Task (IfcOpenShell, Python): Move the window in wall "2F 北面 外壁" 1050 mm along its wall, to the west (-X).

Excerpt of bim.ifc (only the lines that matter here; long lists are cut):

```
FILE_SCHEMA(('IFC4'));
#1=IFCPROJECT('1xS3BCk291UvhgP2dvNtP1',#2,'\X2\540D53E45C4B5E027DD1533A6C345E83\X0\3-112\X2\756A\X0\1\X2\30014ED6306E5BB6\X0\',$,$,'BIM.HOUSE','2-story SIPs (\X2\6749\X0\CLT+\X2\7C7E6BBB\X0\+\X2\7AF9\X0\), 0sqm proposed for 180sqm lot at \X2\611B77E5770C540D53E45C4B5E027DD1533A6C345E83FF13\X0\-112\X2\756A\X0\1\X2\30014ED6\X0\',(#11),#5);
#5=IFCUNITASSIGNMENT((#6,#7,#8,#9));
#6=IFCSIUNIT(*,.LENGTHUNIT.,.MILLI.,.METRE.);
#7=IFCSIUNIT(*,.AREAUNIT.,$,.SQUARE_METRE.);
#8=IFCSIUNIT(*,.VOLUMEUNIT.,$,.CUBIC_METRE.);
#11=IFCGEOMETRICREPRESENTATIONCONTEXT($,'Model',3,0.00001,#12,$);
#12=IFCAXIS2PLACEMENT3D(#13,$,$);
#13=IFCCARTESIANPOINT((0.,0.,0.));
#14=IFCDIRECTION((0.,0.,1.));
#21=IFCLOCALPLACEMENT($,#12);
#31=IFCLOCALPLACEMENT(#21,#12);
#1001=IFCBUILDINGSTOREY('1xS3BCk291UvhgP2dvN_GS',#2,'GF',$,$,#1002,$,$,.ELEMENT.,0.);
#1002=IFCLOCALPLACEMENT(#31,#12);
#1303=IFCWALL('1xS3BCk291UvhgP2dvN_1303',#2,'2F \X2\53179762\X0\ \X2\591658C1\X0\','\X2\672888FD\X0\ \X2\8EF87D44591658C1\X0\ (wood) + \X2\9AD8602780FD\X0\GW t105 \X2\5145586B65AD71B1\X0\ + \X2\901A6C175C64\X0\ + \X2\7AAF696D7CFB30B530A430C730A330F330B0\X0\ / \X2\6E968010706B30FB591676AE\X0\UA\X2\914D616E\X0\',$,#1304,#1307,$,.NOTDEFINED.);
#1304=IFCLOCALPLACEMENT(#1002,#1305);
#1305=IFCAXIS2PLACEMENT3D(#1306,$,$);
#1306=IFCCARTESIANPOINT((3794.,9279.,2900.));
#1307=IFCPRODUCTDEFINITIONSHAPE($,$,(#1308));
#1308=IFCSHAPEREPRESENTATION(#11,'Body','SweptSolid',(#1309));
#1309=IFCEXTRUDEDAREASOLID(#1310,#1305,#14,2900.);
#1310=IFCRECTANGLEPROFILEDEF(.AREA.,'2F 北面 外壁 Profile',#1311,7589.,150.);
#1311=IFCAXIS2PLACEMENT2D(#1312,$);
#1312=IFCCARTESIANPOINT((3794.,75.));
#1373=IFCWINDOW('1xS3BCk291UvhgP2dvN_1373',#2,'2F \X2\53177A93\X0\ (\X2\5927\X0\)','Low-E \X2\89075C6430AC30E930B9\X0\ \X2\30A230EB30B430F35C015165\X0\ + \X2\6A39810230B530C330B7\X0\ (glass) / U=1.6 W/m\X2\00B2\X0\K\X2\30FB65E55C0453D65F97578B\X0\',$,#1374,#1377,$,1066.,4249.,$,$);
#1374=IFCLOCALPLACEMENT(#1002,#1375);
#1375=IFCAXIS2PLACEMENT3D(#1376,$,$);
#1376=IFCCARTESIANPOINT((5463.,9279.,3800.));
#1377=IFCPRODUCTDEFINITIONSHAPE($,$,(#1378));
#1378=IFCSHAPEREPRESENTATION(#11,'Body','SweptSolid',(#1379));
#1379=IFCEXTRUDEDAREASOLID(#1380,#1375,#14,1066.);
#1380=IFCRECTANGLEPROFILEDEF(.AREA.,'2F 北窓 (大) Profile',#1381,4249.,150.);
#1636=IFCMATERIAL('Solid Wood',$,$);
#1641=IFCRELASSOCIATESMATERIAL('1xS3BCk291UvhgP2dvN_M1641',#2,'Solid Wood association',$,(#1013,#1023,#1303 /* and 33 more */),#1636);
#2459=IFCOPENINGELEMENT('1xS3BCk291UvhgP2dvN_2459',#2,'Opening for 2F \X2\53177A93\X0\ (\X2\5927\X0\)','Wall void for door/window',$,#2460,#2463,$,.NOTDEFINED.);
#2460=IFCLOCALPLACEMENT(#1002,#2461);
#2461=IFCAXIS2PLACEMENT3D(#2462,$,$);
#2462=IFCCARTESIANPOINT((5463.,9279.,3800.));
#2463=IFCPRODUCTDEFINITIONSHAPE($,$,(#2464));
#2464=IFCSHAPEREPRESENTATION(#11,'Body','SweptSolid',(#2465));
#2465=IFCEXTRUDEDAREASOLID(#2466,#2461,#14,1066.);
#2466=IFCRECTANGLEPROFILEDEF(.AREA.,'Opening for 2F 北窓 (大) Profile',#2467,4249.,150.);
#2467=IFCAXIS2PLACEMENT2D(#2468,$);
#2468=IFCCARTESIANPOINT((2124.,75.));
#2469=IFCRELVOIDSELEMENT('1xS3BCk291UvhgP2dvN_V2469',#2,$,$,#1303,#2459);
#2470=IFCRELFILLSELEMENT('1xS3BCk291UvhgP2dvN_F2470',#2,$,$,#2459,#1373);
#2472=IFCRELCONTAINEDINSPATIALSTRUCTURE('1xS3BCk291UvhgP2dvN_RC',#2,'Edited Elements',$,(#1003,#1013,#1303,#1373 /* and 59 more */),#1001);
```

```python
import ifcopenshell
import ifcopenshell.api.geometry
import ifcopenshell.util.placement

model = ifcopenshell.open("bim.ifc")

window = model.by_id(1373)
opening = window.FillsVoids[0].RelatingOpeningElement
wall = opening.VoidsElements[0].RelatingBuildingElement

wall_matrix = ifcopenshell.util.placement.get_local_placement(wall.ObjectPlacement)
shift = wall_matrix[:3, 0] * -1050.0
before = ifcopenshell.util.placement.get_local_placement(window.ObjectPlacement)[:3, 3].copy()

# The window is not placed relative to its opening, so move both.
for product in (opening, window):
    matrix = ifcopenshell.util.placement.get_local_placement(product.ObjectPlacement)
    matrix[:3, 3] += shift
    ifcopenshell.api.geometry.edit_object_placement(model, product=product, matrix=matrix, is_si=False)

after = ifcopenshell.util.placement.get_local_placement(window.ObjectPlacement)[:3, 3]
print("window moved by", (after - before).round(3) + 0.0)

model.write("bim_v2.ifc")
```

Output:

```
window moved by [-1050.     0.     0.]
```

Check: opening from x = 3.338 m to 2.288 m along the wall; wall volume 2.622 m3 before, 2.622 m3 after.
